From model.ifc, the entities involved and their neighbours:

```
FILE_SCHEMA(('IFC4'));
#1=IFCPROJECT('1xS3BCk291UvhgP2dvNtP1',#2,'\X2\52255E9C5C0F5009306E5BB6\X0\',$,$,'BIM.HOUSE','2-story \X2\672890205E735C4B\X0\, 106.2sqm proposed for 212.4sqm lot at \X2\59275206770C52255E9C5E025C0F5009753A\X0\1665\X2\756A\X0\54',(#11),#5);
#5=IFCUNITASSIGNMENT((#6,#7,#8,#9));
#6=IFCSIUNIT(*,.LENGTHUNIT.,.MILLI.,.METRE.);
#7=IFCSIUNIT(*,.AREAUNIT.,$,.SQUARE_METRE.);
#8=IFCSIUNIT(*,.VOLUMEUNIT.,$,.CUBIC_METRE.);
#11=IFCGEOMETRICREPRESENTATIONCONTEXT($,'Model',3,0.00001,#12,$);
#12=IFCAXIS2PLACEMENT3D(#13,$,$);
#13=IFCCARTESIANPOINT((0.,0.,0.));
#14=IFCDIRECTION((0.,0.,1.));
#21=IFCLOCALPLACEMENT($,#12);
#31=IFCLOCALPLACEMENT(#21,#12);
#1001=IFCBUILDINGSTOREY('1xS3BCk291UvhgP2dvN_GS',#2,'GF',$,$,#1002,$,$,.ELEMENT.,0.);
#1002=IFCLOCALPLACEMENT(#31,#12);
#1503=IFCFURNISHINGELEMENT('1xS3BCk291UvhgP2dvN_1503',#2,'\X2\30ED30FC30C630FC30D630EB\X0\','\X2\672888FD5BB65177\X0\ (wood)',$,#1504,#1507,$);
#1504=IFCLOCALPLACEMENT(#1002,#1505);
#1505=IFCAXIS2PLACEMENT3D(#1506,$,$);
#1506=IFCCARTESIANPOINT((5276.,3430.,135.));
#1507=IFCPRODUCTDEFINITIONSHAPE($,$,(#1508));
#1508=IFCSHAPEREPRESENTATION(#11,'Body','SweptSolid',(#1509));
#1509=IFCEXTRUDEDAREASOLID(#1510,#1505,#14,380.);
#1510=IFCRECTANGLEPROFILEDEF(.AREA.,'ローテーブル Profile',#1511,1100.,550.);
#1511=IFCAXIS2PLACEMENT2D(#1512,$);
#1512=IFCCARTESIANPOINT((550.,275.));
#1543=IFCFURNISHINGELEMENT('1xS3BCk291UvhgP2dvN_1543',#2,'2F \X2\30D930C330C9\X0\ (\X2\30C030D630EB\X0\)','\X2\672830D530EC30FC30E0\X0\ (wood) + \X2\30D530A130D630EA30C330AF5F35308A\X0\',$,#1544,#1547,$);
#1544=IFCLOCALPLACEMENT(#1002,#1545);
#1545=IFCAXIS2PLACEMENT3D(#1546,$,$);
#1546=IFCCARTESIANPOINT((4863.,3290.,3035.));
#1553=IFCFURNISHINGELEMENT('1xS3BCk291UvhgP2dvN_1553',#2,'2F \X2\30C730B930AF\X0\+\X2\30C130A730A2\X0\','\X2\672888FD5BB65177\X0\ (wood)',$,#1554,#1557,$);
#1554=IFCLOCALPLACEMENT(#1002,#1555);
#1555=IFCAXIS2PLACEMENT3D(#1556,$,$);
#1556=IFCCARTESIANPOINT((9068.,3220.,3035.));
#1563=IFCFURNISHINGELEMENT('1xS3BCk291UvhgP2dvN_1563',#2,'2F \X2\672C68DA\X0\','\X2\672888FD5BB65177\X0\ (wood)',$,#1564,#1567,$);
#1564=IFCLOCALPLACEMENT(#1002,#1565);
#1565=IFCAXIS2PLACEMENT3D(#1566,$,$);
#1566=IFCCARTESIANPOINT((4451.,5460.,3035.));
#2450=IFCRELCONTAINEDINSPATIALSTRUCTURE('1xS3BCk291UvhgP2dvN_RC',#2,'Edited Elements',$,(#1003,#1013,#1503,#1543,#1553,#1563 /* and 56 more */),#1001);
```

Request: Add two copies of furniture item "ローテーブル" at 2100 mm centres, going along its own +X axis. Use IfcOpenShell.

```python
import ifcopenshell
import ifcopenshell.api.geometry
import ifcopenshell.api.root
import ifcopenshell.util.element
import ifcopenshell.util.placement
import ifcopenshell.util.unit

model = ifcopenshell.open("model.ifc")
unit_scale = ifcopenshell.util.unit.calculate_unit_scale(model)


def reuse_history(source, copy):
    """copy_class also copies each property set's owner history, people and application; keep the originals."""
    for rel in copy.IsDefinedBy:
        if rel.is_a("IfcRelDefinesByProperties") and (history := rel.RelatingPropertyDefinition.OwnerHistory):
            rel.RelatingPropertyDefinition.OwnerHistory = source.OwnerHistory
            ifcopenshell.util.element.remove_deep2(model, history)


source = model.by_id(1503)
base = ifcopenshell.util.placement.get_local_placement(source.ObjectPlacement)
step = base[:3, 0] * 2.1 / unit_scale

for i in range(1, 3):
    copy = ifcopenshell.api.root.copy_class(model, product=source)
    copy.Representation = ifcopenshell.util.element.copy_deep(
        model, source.Representation, exclude=["IfcGeometricRepresentationContext", "IfcRepresentationMap"]
    )
    reuse_history(source, copy)
    matrix = base.copy()
    matrix[:3, 3] += i * step
    print("added at", matrix[:3, 3].round(3) + 0.0)
    ifcopenshell.api.geometry.edit_object_placement(model, product=copy, matrix=matrix, is_si=False)

model.write("model_v2.ifc")
```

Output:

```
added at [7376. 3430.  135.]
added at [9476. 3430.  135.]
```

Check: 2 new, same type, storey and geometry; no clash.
